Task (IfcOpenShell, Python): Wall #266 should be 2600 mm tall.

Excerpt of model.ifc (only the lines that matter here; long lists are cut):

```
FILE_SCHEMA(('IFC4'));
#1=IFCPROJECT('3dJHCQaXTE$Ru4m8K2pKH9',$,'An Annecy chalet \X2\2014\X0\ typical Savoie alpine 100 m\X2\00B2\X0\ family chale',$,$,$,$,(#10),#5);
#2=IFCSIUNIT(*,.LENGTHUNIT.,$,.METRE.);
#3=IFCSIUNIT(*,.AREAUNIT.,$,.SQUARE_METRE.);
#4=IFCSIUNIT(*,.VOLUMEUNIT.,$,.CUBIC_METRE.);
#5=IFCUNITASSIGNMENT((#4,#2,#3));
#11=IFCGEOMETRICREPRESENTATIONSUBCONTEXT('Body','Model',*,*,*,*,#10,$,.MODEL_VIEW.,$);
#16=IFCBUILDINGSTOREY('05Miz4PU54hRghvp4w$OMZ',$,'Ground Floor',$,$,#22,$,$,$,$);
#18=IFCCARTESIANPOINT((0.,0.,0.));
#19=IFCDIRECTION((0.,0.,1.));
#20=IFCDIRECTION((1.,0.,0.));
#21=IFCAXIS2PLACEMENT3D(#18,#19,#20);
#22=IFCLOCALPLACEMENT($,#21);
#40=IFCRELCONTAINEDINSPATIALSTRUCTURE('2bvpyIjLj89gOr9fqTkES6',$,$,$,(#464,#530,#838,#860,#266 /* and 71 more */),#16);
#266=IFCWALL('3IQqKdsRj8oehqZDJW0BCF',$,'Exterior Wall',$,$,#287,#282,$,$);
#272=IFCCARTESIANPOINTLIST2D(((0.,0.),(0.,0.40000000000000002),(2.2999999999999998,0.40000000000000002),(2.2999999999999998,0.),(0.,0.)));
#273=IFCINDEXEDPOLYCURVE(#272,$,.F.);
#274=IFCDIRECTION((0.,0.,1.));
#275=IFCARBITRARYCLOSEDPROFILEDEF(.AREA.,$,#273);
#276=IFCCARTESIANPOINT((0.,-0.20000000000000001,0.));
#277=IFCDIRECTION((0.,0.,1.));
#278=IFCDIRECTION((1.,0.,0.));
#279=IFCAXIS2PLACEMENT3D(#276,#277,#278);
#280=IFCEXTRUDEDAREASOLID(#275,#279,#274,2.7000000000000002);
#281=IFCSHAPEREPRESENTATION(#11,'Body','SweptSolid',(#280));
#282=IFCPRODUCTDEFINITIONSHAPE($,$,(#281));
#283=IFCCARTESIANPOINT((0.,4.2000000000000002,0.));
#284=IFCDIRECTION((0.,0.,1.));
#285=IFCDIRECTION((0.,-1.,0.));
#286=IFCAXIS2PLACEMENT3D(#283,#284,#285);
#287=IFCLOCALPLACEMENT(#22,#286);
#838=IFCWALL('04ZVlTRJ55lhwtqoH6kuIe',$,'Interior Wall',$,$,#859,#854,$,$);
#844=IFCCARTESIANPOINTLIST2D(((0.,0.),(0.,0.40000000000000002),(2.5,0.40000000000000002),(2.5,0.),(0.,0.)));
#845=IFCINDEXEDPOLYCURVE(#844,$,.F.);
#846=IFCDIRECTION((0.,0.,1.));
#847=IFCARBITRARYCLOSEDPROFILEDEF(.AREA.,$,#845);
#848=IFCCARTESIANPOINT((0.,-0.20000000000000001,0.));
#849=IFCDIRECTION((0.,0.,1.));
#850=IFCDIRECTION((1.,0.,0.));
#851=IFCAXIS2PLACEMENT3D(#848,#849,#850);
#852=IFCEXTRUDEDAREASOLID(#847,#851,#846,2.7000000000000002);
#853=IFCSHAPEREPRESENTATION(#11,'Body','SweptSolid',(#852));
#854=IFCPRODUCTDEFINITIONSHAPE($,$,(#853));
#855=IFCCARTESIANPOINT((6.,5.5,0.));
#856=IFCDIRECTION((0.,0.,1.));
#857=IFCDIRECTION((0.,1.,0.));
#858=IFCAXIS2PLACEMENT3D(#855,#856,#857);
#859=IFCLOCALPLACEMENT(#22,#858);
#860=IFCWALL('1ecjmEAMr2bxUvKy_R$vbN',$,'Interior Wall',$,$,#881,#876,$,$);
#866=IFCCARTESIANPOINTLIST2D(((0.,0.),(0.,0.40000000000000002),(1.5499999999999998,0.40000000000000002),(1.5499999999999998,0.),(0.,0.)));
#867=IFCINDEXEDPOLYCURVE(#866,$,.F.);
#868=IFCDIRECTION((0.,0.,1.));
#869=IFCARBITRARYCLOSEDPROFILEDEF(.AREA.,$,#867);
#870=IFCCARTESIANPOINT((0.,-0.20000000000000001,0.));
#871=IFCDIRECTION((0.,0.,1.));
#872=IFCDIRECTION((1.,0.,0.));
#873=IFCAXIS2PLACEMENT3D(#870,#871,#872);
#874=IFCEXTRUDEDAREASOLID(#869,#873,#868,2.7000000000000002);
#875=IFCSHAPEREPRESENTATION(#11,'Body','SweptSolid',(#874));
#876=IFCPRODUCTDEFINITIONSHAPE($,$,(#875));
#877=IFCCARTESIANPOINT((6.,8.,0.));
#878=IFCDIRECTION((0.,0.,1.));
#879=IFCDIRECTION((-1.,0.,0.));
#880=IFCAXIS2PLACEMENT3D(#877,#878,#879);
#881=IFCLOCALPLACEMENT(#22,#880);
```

```python
import ifcopenshell
import ifcopenshell.geom
import ifcopenshell.util.representation
import ifcopenshell.util.shape
import ifcopenshell.util.unit

model = ifcopenshell.open("model.ifc")
unit_scale = ifcopenshell.util.unit.calculate_unit_scale(model)
settings = ifcopenshell.geom.settings()


def volume(element):
    """Net volume in cubic metres, openings subtracted."""
    shape = ifcopenshell.geom.create_shape(settings, element)
    return ifcopenshell.util.shape.get_volume(shape.geometry)


wall = model.by_id(266)
before = volume(wall)

body = ifcopenshell.util.representation.get_representation(wall, "Model", "Body")
solid = body.Items[0]
old_height = solid.Depth
solid.Depth = 2.6 / unit_scale
after = volume(wall)

print(f"height {old_height:g} -> {solid.Depth:g}, volume {before:.3f} -> {after:.3f} m3")

model.write("model_updated.ifc")
```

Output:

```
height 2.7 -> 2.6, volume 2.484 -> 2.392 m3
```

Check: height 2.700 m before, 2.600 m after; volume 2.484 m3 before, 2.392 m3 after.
